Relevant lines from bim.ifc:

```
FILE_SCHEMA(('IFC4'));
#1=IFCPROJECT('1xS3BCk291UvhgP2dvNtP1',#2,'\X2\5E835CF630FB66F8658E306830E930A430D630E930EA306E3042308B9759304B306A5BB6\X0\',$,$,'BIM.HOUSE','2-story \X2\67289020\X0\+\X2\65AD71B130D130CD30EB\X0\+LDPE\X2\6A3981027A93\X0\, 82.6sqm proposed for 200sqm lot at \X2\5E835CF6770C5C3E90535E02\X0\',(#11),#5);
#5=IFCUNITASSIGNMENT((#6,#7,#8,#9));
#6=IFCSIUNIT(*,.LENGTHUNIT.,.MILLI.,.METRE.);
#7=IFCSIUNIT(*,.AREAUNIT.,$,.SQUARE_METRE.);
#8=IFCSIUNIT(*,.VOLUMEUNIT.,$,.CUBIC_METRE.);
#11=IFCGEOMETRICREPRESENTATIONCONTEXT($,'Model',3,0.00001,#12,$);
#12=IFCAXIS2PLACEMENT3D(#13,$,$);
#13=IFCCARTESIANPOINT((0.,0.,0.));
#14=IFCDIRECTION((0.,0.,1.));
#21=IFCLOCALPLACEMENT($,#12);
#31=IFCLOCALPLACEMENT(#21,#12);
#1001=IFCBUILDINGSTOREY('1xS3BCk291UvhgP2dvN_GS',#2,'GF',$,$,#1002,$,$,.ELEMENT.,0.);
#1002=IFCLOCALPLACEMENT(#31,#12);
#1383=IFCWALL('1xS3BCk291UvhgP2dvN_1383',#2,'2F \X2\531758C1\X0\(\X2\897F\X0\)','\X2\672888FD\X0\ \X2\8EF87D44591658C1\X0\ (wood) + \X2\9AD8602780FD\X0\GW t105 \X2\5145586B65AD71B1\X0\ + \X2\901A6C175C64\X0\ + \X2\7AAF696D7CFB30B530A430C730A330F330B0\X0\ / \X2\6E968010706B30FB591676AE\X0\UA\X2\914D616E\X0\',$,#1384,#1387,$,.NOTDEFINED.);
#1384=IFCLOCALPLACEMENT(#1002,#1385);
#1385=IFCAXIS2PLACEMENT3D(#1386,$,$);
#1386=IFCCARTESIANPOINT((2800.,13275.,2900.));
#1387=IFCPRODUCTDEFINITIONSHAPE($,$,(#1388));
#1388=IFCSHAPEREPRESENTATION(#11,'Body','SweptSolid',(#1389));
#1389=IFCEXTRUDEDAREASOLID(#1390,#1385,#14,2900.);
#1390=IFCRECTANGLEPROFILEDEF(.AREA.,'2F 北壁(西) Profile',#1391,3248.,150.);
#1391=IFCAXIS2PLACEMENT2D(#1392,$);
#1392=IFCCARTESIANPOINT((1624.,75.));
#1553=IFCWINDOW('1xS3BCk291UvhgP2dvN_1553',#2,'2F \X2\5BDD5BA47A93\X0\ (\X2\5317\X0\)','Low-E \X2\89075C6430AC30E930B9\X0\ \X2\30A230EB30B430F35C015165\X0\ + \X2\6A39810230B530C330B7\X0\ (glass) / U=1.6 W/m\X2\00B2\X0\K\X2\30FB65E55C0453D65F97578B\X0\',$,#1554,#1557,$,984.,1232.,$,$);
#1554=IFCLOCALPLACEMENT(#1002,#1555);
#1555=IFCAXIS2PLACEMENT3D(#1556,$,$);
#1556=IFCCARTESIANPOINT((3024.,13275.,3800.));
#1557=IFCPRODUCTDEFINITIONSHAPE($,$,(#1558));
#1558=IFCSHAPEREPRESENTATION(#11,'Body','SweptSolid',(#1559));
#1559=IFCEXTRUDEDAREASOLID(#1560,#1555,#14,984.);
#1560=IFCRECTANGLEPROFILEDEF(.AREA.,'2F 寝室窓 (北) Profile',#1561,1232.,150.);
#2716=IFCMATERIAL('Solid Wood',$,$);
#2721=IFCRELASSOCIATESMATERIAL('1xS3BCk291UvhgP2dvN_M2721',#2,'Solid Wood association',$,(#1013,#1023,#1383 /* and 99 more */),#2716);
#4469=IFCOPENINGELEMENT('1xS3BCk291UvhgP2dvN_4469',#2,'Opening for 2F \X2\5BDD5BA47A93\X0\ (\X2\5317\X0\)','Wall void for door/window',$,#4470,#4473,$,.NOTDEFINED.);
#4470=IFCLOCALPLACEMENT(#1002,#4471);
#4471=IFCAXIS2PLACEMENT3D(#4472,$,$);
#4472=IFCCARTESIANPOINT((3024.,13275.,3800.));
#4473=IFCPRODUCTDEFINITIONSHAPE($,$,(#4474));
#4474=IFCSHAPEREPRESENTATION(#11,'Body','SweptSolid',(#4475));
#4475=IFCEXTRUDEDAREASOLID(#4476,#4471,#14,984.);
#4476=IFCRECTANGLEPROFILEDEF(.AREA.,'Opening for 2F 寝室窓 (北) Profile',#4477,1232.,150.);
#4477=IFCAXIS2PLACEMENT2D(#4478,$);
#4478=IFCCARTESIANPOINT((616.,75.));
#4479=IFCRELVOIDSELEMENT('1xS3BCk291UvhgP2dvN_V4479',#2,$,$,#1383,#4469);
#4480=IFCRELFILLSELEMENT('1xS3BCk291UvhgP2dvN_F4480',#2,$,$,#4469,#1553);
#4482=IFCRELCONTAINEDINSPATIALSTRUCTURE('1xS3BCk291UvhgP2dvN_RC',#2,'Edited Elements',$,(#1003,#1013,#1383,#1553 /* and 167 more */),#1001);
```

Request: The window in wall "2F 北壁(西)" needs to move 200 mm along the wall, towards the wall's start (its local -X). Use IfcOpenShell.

```python
import ifcopenshell
import ifcopenshell.api.geometry
import ifcopenshell.util.placement
import ifcopenshell.util.unit

model = ifcopenshell.open("bim.ifc")
unit_scale = ifcopenshell.util.unit.calculate_unit_scale(model)

window = model.by_guid("1xS3BCk291UvhgP2dvN_1553")
opening = window.FillsVoids[0].RelatingOpeningElement
wall = opening.VoidsElements[0].RelatingBuildingElement

wall_matrix = ifcopenshell.util.placement.get_local_placement(wall.ObjectPlacement)
shift = wall_matrix[:3, 0] * -0.2 / unit_scale
before = ifcopenshell.util.placement.get_local_placement(window.ObjectPlacement)[:3, 3].copy()

# The window is not placed relative to its opening, so move both.
for product in (opening, window):
    matrix = ifcopenshell.util.placement.get_local_placement(product.ObjectPlacement)
    matrix[:3, 3] += shift
    ifcopenshell.api.geometry.edit_object_placement(model, product=product, matrix=matrix, is_si=False)

after = ifcopenshell.util.placement.get_local_placement(window.ObjectPlacement)[:3, 3]
print("window moved by", (after - before).round(3) + 0.0)

model.write("bim_updated.ifc")
```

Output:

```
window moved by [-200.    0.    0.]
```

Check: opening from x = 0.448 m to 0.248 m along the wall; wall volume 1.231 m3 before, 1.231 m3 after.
